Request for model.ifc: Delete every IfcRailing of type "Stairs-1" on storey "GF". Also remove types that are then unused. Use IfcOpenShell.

First a look at what the model holds.

```python
import ifcopenshell
import ifcopenshell.util.element

model = ifcopenshell.open("model.ifc")
print(model.schema)
storey = next(s for s in model.by_type("IfcBuildingStorey") if s.Name == "GF")
railings = [e for e in ifcopenshell.util.element.get_decomposition(storey) if e.is_a("IfcRailing")]
seen = {}
for e in railings:
    element_type = ifcopenshell.util.element.get_type(e)
    name = element_type.Name if element_type not in (None, e) else None
    seen[name] = seen.get(name, 0) + 1
for name, count in sorted(seen.items(), key=str):
    print(count, "x", name)
```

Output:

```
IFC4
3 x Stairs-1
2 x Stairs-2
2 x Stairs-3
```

```python
import ifcopenshell
import ifcopenshell.api.root
import ifcopenshell.util.element

model = ifcopenshell.open("model.ifc")

storey = next(s for s in model.by_type("IfcBuildingStorey") if s.Name == "GF")
railings = [e for e in ifcopenshell.util.element.get_decomposition(storey) if e.is_a("IfcRailing")]
targets = [e for e in railings if (t := ifcopenshell.util.element.get_type(e)) not in (None, e) and t.Name == "Stairs-1"]
types = {ifcopenshell.util.element.get_type(e) for e in targets} - {None, *targets}

for e in targets:
    ifcopenshell.api.root.remove_product(model, product=e)
print(len(targets), "removed")

unused = [t for t in types if not ifcopenshell.util.element.get_types(t)]
for t in unused:
    ifcopenshell.api.root.remove_product(model, product=t)
print(len(unused), "unused types removed")

model.write("model_rev.ifc")
```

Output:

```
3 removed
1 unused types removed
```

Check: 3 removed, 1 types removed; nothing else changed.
